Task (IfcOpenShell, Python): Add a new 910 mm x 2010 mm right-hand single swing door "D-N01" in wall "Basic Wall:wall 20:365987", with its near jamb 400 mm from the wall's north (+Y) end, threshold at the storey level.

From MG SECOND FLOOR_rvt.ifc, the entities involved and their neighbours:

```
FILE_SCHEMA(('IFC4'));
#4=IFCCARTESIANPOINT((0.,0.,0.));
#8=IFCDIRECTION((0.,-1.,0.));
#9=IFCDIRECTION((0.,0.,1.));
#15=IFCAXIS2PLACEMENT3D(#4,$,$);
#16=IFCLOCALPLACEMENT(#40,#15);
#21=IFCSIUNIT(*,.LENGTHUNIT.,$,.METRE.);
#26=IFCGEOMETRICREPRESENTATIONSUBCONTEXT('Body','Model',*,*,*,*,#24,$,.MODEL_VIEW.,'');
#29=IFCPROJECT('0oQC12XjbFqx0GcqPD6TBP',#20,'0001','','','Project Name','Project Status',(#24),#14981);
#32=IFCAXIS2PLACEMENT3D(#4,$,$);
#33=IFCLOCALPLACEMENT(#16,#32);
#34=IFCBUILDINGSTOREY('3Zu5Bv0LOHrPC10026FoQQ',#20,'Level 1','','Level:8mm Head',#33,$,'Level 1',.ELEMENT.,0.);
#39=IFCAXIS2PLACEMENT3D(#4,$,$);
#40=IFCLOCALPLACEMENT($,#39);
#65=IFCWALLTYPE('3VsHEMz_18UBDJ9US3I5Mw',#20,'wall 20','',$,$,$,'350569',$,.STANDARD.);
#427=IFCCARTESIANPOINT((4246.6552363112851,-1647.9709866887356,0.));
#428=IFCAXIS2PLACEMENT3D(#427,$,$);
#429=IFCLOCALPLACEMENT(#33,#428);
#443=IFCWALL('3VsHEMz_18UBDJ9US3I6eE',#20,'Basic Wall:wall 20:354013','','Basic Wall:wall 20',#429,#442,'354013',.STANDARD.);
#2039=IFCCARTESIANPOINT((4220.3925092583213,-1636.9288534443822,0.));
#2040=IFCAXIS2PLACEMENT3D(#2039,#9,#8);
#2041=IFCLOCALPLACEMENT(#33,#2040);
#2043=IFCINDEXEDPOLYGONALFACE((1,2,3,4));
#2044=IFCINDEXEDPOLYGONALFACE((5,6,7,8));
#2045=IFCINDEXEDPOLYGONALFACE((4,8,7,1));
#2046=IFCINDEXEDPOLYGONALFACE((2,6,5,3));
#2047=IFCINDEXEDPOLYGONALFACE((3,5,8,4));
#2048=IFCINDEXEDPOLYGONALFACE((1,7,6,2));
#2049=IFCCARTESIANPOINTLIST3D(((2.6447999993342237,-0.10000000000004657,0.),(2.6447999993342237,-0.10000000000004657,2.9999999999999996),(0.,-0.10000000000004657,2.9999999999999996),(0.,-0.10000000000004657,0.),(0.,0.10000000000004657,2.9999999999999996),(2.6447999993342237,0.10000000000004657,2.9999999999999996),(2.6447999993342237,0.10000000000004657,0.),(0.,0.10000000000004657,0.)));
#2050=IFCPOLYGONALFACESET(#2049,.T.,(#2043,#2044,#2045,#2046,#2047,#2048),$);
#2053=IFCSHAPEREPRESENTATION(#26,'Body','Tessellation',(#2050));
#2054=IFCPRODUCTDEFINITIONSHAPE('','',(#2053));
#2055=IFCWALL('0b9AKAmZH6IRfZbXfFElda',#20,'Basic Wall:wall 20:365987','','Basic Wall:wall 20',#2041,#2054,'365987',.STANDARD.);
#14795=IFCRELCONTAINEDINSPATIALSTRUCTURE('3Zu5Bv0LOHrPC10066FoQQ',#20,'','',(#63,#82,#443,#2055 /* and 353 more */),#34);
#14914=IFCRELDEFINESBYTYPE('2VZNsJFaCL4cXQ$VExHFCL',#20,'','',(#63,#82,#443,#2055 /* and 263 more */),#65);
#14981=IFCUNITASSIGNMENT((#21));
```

```python
import numpy as np
import ifcopenshell
import ifcopenshell.api.feature
import ifcopenshell.api.geometry
import ifcopenshell.api.root
import ifcopenshell.api.spatial
import ifcopenshell.geom
import ifcopenshell.util.element
import ifcopenshell.util.placement
import ifcopenshell.util.representation
import ifcopenshell.util.shape
import ifcopenshell.util.unit

model = ifcopenshell.open("MG SECOND FLOOR_rvt.ifc")
unit_scale = ifcopenshell.util.unit.calculate_unit_scale(model)
settings = ifcopenshell.geom.settings()


def volume(element):
    """Net volume in cubic metres, openings subtracted."""
    shape = ifcopenshell.geom.create_shape(settings, element)
    return ifcopenshell.util.shape.get_volume(shape.geometry)


wall = model.by_guid("0b9AKAmZH6IRfZbXfFElda")
storey = ifcopenshell.util.element.get_container(wall, ifc_class="IfcBuildingStorey")
context = ifcopenshell.util.representation.get_context(model, "Model", "Body", "MODEL_VIEW")
before = volume(wall)

width, height, from_end, sill = 0.91, 2.01, 0.4, 0.0  # metres

# The wall runs along its own X axis, and the end named is its -X end.
wall_shape = ifcopenshell.geom.create_shape(settings, wall)
x, y, z = ifcopenshell.util.shape.get_vertices(wall_shape.geometry).T
start = x.min() + from_end
face, thickness = float(y.min()), float(y.max() - y.min())
wall_matrix = ifcopenshell.util.placement.get_local_placement(wall.ObjectPlacement)
level = ifcopenshell.util.placement.get_local_placement(storey.ObjectPlacement)[2, 3]


def in_wall(x, y):
    """Placement at x, y metres in the wall's axes, at sill height."""
    matrix = wall_matrix.copy()
    matrix[:, 3] = wall_matrix @ np.array([x / unit_scale, y / unit_scale, 0.0, 1.0])
    matrix[2, 3] = level + sill / unit_scale
    return matrix


# Opening: a box that overshoots both wall faces by 50 mm.
opening = ifcopenshell.api.root.create_entity(model, ifc_class="IfcOpeningElement", predefined_type="OPENING")
box = ifcopenshell.api.geometry.add_wall_representation(
    model, context=context, length=width, height=height, thickness=thickness + 0.1
)
ifcopenshell.api.geometry.assign_representation(model, product=opening, representation=box)
ifcopenshell.api.geometry.edit_object_placement(model, product=opening, matrix=in_wall(start, face - 0.05), is_si=False)
ifcopenshell.api.feature.add_feature(model, feature=opening, element=wall)

door = ifcopenshell.api.root.create_entity(model, ifc_class="IfcDoor", name="D-N01", predefined_type="DOOR")
door.OverallWidth, door.OverallHeight = width / unit_scale, height / unit_scale
door.OperationType = "SINGLE_SWING_RIGHT"
body = ifcopenshell.api.geometry.add_door_representation(
    model,
    context=context,
    overall_width=door.OverallWidth,
    overall_height=door.OverallHeight,
    operation_type="SINGLE_SWING_RIGHT",
    lining_properties={"LiningDepth": thickness / unit_scale, "ThresholdDepth": thickness / unit_scale},
)
ifcopenshell.api.geometry.assign_representation(model, product=door, representation=body)
ifcopenshell.api.spatial.assign_container(model, products=[door], relating_structure=storey)
ifcopenshell.api.feature.add_filling(model, opening=opening, element=door)

# The lining spans the wall, so the door starts at the wall face.
ifcopenshell.api.geometry.edit_object_placement(model, product=door, matrix=in_wall(start, face), is_si=False)

after = volume(wall)

print(f"wall volume {before:.3f} -> {after:.3f} m3")

model.write("MG SECOND FLOOR_rvt_rev.ifc")
```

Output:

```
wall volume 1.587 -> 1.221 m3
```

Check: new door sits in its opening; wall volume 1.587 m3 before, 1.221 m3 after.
